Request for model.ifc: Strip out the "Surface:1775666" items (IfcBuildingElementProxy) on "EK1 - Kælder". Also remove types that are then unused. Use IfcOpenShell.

First a look at what the model holds.

```python
import ifcopenshell
import ifcopenshell.util.element

model = ifcopenshell.open("model.ifc")
print(model.schema)
storey = next(s for s in model.by_type("IfcBuildingStorey") if s.Name == "EK1 - Kælder")
proxies = [e for e in ifcopenshell.util.element.get_decomposition(storey) if e.is_a("IfcBuildingElementProxy")]
seen = {}
for e in proxies:
    element_type = ifcopenshell.util.element.get_type(e)
    name = element_type.Name if element_type not in (None, e) else None
    seen[name] = seen.get(name, 0) + 1
for name, count in sorted(seen.items(), key=str):
    print(count, "x", name)
```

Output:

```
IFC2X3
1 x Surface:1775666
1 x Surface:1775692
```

```python
import ifcopenshell
import ifcopenshell.api.root
import ifcopenshell.util.element

model = ifcopenshell.open("model.ifc")

storey = next(s for s in model.by_type("IfcBuildingStorey") if s.Name == "EK1 - Kælder")
proxies = [e for e in ifcopenshell.util.element.get_decomposition(storey) if e.is_a("IfcBuildingElementProxy")]
targets = [e for e in proxies if (t := ifcopenshell.util.element.get_type(e)) not in (None, e) and t.Name == "Surface:1775666"]
types = {ifcopenshell.util.element.get_type(e) for e in targets} - {None, *targets}

for e in targets:
    ifcopenshell.api.root.remove_product(model, product=e)
print(len(targets), "removed")

unused = [t for t in types if not ifcopenshell.util.element.get_types(t)]
for t in unused:
    ifcopenshell.api.root.remove_product(model, product=t)
print(len(unused), "unused types removed")

model.write("model_edited.ifc")
```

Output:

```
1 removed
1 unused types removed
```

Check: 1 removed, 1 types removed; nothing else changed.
